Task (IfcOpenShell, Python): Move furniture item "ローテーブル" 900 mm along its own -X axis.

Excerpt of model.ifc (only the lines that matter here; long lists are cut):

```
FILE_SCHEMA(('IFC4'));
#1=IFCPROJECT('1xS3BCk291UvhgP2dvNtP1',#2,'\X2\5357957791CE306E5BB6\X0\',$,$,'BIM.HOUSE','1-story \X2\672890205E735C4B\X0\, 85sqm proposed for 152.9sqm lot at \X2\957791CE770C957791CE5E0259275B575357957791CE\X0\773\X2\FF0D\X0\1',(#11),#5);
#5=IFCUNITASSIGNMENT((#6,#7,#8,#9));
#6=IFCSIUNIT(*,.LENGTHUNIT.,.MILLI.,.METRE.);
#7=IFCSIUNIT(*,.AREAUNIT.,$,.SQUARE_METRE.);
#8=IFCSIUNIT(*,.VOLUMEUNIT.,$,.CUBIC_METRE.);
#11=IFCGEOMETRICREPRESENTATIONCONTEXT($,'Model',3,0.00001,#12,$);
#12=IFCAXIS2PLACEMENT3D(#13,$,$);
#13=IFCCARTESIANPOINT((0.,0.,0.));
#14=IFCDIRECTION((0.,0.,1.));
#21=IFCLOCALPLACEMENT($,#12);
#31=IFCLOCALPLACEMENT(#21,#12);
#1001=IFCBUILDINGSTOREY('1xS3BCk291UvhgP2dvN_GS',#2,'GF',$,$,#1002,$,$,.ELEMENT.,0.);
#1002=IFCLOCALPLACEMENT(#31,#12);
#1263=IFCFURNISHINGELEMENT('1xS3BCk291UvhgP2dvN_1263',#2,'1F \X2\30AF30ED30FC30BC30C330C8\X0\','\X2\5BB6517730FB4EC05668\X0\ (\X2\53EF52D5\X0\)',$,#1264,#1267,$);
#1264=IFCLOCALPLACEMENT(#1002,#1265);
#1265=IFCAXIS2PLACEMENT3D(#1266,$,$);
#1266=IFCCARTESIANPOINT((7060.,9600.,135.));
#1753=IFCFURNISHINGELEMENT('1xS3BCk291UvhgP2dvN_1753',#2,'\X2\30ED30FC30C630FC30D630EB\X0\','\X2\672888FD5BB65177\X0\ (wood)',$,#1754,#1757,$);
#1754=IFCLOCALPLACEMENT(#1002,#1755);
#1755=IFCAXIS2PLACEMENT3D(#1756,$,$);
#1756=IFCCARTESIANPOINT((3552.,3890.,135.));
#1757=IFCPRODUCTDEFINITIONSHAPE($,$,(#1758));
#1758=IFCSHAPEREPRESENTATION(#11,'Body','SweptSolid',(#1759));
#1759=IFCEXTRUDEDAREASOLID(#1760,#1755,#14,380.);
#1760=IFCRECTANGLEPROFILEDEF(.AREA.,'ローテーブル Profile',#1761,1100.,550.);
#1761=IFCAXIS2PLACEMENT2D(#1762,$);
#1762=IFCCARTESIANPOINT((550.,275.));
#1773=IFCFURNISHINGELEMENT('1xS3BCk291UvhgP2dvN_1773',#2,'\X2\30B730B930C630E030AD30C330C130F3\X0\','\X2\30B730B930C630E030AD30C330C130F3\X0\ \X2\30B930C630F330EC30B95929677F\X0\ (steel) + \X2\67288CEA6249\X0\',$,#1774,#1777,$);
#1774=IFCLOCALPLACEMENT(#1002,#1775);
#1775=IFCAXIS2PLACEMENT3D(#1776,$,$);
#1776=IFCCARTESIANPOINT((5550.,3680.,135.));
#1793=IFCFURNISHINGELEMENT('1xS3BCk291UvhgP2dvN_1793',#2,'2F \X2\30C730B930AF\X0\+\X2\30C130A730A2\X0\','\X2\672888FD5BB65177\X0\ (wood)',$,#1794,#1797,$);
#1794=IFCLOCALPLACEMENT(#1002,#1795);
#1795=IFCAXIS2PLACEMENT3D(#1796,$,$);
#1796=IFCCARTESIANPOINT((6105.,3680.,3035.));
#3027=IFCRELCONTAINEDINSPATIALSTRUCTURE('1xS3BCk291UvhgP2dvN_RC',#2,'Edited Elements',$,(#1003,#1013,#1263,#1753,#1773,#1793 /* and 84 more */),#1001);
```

```python
import ifcopenshell
import ifcopenshell.api.geometry
import ifcopenshell.util.placement
import ifcopenshell.util.unit

model = ifcopenshell.open("model.ifc")
unit_scale = ifcopenshell.util.unit.calculate_unit_scale(model)

item = model.by_guid("1xS3BCk291UvhgP2dvN_1753")
matrix = ifcopenshell.util.placement.get_local_placement(item.ObjectPlacement)
matrix[:3, 3] -= matrix[:3, 0] * 0.9 / unit_scale
ifcopenshell.api.geometry.edit_object_placement(model, product=item, matrix=matrix, is_si=False)

print(ifcopenshell.util.placement.get_local_placement(item.ObjectPlacement).round(3) + 0.0)

model.write("model_rev.ifc")
```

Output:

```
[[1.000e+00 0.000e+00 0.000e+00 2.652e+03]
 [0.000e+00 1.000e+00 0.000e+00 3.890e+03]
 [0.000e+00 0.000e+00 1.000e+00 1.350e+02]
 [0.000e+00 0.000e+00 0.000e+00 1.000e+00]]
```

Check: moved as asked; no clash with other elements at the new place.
